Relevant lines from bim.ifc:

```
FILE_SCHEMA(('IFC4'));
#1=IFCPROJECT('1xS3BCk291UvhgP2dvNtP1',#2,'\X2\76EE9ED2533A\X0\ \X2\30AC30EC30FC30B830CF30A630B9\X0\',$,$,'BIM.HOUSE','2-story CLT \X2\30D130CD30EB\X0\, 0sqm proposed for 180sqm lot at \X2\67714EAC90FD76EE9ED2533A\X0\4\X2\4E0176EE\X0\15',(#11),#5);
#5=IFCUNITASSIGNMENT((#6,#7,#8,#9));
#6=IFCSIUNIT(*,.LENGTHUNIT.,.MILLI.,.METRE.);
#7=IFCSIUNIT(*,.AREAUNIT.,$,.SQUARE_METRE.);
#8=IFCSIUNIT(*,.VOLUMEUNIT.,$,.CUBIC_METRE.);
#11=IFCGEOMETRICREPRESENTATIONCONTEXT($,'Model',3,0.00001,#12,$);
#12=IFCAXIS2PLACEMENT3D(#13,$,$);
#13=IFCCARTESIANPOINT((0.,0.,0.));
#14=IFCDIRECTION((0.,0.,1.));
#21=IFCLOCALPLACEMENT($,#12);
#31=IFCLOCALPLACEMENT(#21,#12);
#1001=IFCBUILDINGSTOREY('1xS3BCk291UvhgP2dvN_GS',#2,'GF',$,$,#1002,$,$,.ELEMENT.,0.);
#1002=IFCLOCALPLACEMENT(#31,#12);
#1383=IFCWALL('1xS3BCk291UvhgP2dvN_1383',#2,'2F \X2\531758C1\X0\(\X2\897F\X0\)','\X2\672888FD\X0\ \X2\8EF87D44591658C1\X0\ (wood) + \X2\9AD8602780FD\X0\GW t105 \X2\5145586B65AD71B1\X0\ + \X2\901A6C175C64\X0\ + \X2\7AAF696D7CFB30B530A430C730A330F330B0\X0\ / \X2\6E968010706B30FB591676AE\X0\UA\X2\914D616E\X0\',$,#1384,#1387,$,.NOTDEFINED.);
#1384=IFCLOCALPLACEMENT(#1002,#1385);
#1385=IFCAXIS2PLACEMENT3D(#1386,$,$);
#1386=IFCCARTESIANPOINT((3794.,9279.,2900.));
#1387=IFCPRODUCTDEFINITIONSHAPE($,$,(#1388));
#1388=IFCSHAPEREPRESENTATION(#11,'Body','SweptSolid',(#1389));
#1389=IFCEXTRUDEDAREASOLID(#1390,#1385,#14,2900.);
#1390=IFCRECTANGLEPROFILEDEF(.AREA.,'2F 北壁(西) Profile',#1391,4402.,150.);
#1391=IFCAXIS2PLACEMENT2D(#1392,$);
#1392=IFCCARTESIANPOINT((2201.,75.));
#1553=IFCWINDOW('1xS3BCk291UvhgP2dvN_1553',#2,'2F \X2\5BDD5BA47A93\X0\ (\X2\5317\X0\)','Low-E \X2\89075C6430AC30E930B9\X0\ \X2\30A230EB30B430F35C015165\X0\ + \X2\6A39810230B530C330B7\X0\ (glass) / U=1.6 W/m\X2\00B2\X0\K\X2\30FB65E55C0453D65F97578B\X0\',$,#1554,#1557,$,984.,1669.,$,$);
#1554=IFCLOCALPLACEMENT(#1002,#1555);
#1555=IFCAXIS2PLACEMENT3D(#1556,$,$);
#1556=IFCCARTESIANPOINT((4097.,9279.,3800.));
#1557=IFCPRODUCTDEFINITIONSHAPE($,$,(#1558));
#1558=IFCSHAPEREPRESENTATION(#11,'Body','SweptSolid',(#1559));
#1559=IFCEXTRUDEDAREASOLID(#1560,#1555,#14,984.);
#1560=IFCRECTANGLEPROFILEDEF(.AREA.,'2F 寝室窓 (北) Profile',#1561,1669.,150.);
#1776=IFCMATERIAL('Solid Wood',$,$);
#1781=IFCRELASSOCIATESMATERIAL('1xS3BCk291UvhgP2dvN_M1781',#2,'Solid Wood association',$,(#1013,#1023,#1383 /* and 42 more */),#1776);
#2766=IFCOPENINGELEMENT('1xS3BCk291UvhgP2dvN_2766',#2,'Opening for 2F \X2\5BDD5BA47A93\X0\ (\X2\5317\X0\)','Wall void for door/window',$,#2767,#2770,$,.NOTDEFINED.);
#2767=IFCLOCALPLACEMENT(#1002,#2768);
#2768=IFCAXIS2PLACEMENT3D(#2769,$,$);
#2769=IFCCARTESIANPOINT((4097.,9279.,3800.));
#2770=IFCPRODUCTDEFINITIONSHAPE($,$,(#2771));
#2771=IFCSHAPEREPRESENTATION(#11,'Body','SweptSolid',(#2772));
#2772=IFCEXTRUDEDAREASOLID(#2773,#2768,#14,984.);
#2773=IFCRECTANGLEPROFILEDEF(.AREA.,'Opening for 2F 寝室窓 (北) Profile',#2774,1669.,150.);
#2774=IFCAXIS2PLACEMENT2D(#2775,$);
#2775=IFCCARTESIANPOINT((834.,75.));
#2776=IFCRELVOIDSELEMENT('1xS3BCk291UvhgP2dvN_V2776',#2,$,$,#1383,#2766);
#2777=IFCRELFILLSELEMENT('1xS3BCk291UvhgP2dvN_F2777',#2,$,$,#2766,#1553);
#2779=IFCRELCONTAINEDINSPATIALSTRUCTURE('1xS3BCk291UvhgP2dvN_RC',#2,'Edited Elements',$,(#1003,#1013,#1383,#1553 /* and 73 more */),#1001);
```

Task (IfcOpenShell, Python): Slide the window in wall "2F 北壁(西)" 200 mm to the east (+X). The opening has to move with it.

```python
import ifcopenshell
import ifcopenshell.api.geometry
import ifcopenshell.util.placement

model = ifcopenshell.open("bim.ifc")

window = model.by_guid("1xS3BCk291UvhgP2dvN_1553")
opening = window.FillsVoids[0].RelatingOpeningElement
wall = opening.VoidsElements[0].RelatingBuildingElement

wall_matrix = ifcopenshell.util.placement.get_local_placement(wall.ObjectPlacement)
shift = wall_matrix[:3, 0] * 200.0
before = ifcopenshell.util.placement.get_local_placement(window.ObjectPlacement)[:3, 3].copy()

# The window is not placed relative to its opening, so move both.
for product in (opening, window):
    matrix = ifcopenshell.util.placement.get_local_placement(product.ObjectPlacement)
    matrix[:3, 3] += shift
    ifcopenshell.api.geometry.edit_object_placement(model, product=product, matrix=matrix, is_si=False)

after = ifcopenshell.util.placement.get_local_placement(window.ObjectPlacement)[:3, 3]
print("window moved by", (after - before).round(3) + 0.0)

model.write("bim_updated.ifc")
```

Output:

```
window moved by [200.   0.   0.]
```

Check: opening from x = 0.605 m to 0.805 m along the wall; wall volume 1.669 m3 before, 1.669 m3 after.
